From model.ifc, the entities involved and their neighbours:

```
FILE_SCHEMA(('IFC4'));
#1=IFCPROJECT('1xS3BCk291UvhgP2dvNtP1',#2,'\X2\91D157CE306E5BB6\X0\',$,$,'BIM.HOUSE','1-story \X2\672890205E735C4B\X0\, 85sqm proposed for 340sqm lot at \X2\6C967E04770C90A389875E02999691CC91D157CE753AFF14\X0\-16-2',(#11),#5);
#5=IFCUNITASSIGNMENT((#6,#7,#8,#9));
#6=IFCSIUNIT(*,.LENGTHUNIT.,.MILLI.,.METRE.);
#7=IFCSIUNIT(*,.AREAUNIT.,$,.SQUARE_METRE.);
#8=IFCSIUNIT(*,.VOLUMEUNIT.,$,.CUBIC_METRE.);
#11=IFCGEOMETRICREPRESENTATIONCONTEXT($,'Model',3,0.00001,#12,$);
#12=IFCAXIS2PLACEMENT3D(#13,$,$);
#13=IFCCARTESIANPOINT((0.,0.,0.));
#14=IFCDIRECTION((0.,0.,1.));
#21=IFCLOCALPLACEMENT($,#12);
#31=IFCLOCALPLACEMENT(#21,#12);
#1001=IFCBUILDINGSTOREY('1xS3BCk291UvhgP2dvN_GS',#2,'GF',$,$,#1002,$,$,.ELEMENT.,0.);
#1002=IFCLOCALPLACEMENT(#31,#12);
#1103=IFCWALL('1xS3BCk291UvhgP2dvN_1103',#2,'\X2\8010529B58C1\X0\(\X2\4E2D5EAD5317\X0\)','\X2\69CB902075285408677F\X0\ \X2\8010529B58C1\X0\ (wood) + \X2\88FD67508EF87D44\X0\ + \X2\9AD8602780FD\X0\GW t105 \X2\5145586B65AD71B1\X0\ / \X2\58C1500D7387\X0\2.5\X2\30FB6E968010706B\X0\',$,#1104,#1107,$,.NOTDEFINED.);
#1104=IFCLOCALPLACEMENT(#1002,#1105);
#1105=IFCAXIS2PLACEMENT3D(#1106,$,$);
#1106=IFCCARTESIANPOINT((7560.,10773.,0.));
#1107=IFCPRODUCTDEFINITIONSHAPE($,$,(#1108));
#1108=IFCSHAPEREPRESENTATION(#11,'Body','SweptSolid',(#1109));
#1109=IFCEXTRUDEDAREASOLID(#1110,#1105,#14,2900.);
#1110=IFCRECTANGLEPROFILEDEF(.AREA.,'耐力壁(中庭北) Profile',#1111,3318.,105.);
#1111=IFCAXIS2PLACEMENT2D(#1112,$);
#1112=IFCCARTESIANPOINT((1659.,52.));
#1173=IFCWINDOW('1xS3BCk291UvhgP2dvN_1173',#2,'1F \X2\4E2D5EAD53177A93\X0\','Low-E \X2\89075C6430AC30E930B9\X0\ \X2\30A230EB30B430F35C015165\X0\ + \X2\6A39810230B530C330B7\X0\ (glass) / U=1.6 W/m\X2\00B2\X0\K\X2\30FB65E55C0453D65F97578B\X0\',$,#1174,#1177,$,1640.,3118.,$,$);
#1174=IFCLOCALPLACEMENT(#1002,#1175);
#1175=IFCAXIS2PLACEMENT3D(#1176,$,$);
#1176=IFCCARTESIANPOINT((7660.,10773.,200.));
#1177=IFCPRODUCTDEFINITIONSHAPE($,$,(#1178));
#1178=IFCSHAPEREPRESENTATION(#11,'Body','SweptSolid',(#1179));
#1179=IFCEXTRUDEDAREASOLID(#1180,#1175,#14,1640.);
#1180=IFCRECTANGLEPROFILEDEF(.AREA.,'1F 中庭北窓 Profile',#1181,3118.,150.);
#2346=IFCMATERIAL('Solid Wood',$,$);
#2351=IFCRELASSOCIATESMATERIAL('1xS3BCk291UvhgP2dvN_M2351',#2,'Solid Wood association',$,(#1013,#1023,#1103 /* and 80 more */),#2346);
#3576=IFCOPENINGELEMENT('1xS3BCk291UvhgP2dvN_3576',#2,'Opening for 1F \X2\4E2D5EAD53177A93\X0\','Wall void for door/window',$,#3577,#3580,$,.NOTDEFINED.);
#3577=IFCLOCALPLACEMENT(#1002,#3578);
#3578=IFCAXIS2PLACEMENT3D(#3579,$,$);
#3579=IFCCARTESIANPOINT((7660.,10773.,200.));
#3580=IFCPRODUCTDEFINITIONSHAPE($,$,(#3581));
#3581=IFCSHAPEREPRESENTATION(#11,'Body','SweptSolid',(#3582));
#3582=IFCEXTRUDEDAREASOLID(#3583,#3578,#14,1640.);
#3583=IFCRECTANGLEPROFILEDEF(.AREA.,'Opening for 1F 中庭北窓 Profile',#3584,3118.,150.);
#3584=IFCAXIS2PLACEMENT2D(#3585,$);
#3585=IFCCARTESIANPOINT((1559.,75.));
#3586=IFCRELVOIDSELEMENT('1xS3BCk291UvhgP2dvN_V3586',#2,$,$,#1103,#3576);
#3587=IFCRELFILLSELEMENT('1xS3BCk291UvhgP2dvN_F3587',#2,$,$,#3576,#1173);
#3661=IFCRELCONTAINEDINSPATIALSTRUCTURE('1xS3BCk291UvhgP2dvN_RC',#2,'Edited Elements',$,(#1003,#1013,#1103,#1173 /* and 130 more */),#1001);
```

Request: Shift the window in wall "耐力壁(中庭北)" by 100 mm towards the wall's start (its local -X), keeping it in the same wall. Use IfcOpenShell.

```python
import ifcopenshell
import ifcopenshell.api.geometry
import ifcopenshell.util.placement
import ifcopenshell.util.unit

model = ifcopenshell.open("model.ifc")
unit_scale = ifcopenshell.util.unit.calculate_unit_scale(model)

window = model.by_guid("1xS3BCk291UvhgP2dvN_1173")
opening = window.FillsVoids[0].RelatingOpeningElement
wall = opening.VoidsElements[0].RelatingBuildingElement

wall_matrix = ifcopenshell.util.placement.get_local_placement(wall.ObjectPlacement)
shift = wall_matrix[:3, 0] * -0.1 / unit_scale
before = ifcopenshell.util.placement.get_local_placement(window.ObjectPlacement)[:3, 3].copy()

# The window is not placed relative to its opening, so move both.
for product in (opening, window):
    matrix = ifcopenshell.util.placement.get_local_placement(product.ObjectPlacement)
    matrix[:3, 3] += shift
    ifcopenshell.api.geometry.edit_object_placement(model, product=product, matrix=matrix, is_si=False)

after = ifcopenshell.util.placement.get_local_placement(window.ObjectPlacement)[:3, 3]
print("window moved by", (after - before).round(3) + 0.0)

model.write("model_rev.ifc")
```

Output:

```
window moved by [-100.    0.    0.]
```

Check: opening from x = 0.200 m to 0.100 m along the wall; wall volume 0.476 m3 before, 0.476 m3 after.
